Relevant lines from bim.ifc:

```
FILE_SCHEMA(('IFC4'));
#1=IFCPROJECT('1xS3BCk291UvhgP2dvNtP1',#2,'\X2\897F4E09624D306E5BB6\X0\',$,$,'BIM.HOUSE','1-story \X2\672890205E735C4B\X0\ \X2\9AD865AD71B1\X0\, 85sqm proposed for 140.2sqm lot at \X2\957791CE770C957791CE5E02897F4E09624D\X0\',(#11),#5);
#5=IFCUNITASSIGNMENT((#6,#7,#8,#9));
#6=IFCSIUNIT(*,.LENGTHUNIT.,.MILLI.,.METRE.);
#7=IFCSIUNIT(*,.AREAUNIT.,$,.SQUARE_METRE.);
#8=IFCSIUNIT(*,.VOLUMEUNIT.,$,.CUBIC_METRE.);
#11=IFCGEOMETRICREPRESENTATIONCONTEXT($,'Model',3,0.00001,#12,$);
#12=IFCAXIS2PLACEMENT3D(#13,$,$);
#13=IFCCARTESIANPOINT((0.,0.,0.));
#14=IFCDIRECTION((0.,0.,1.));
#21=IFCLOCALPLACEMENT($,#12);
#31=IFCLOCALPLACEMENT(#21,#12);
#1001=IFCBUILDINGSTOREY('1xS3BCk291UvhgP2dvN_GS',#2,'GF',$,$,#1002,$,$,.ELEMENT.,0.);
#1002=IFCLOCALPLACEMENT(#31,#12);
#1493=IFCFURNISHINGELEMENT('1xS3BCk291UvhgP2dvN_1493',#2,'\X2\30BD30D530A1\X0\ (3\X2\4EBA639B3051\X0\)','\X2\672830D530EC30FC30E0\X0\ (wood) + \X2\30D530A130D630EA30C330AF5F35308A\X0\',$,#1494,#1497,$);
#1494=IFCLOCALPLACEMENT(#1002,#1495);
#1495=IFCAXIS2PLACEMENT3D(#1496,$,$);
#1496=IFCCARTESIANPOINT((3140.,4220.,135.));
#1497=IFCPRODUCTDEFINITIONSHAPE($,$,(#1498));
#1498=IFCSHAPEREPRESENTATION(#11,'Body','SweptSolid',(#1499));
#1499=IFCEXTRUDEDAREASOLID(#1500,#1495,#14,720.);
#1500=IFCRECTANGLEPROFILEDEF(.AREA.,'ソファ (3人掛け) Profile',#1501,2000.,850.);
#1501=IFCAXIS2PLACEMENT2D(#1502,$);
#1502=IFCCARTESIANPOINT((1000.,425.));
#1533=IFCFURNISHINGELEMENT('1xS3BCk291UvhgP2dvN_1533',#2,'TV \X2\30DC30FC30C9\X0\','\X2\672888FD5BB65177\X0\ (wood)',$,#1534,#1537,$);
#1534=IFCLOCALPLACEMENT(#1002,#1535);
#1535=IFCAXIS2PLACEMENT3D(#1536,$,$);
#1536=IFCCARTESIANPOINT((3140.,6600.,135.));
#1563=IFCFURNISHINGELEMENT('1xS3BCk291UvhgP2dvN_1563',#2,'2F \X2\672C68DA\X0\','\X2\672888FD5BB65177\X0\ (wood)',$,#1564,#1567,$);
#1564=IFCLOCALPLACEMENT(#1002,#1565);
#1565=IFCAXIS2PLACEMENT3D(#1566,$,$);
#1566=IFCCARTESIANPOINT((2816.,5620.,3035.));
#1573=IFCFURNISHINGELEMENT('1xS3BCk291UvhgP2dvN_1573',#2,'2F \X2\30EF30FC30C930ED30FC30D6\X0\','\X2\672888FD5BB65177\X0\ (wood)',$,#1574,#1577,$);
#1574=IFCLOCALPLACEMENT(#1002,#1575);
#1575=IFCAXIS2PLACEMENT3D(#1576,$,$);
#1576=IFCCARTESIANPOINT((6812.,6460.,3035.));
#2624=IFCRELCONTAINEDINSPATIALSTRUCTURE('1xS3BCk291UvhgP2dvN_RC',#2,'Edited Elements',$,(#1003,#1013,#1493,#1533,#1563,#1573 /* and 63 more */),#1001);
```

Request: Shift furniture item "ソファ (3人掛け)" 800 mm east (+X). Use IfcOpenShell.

```python
import ifcopenshell
import ifcopenshell.api.geometry
import ifcopenshell.util.placement

model = ifcopenshell.open("bim.ifc")

item = model.by_guid("1xS3BCk291UvhgP2dvN_1493")
matrix = ifcopenshell.util.placement.get_local_placement(item.ObjectPlacement)
matrix[0, 3] += 800.0
ifcopenshell.api.geometry.edit_object_placement(model, product=item, matrix=matrix, is_si=False)

print(ifcopenshell.util.placement.get_local_placement(item.ObjectPlacement).round(3) + 0.0)

model.write("bim_edited.ifc")
```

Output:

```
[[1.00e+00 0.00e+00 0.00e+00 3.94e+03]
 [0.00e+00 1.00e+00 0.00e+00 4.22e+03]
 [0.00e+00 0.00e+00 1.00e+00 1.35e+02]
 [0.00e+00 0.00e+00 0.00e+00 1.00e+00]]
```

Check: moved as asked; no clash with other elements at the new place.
